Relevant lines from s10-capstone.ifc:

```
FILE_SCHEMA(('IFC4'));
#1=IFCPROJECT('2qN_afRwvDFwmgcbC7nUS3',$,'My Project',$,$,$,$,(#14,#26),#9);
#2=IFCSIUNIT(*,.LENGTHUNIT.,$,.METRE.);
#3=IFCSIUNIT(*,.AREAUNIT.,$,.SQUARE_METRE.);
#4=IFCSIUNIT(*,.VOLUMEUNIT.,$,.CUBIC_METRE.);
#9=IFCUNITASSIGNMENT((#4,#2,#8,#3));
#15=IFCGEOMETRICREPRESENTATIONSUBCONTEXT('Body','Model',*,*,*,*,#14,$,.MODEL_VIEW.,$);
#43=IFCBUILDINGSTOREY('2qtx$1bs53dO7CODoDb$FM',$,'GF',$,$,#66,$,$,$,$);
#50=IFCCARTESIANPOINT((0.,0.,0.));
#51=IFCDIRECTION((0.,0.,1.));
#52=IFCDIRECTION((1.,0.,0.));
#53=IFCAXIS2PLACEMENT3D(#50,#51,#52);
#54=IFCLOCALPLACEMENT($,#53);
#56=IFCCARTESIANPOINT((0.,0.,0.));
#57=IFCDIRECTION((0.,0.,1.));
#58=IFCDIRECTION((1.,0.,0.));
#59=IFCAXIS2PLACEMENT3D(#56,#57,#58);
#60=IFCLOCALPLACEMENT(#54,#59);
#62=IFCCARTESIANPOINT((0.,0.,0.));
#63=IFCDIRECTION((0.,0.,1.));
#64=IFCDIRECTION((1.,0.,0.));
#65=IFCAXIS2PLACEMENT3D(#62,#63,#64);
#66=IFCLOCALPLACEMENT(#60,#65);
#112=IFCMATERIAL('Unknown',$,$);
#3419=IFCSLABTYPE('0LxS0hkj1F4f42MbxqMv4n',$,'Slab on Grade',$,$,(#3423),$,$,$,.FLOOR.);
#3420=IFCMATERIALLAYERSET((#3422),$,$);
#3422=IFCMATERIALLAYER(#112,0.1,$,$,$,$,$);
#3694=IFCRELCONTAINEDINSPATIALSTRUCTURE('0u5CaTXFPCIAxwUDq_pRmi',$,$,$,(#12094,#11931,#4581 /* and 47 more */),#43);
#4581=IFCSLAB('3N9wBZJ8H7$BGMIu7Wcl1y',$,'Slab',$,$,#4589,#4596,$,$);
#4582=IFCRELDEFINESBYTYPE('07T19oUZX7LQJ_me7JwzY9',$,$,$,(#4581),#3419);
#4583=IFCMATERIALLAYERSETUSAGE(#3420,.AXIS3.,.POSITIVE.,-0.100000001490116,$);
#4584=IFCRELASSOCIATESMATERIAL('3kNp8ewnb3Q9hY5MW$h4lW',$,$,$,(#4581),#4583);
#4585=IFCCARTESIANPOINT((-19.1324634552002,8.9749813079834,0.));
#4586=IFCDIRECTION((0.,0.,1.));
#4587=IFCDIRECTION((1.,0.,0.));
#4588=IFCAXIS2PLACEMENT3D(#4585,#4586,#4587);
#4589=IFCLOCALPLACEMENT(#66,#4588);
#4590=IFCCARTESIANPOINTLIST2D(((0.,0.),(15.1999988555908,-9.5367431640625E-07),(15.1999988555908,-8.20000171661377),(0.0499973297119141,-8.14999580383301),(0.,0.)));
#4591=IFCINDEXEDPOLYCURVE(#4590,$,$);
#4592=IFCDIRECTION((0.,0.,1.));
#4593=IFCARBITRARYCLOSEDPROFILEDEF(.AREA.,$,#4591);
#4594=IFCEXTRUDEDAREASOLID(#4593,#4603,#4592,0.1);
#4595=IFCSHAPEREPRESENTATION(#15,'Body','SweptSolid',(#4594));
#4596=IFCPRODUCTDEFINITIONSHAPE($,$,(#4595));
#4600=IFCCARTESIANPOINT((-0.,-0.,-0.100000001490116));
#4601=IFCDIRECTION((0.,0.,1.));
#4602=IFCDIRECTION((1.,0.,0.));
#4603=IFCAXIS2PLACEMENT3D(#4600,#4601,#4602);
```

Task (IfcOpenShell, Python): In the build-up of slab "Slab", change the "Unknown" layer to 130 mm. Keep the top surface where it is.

```python
import ifcopenshell
import ifcopenshell.util.element
import ifcopenshell.util.representation
import ifcopenshell.util.unit

model = ifcopenshell.open("s10-capstone.ifc")
unit_scale = ifcopenshell.util.unit.calculate_unit_scale(model)

layer_set = model.by_id(3420)
layer = next(l for l in layer_set.MaterialLayers if l.Material and l.Material.Name == "Unknown")
change = 0.13 / unit_scale - layer.LayerThickness
layer.LayerThickness += change

# Geometry does not follow the layer set by itself.
slabs = [e for e in ifcopenshell.util.element.get_elements_by_material(model, layer_set) if e.is_a("IfcSlab")]
for slab in sorted(slabs, key=lambda e: e.id()):
    body = ifcopenshell.util.representation.get_representation(slab, "Model", "Body")
    solid = body.Items[0]
    old_depth = solid.Depth
    solid.Depth += change
    # Extruded upwards: lower the start of the extrusion so the top stays.
    x, y, z = solid.Position.Location.Coordinates
    solid.Position.Location = model.createIfcCartesianPoint((x, y, z - change))
    print(slab.id(), f"{old_depth:g} -> {solid.Depth:g}")

# The layers are counted up from the underside, which has moved.
for usage in {ifcopenshell.util.element.get_material(slab) for slab in slabs}:
    usage.OffsetFromReferenceLine -= change

model.write("s10-capstone_rev.ifc")
```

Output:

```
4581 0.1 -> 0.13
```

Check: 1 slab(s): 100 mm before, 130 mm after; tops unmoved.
